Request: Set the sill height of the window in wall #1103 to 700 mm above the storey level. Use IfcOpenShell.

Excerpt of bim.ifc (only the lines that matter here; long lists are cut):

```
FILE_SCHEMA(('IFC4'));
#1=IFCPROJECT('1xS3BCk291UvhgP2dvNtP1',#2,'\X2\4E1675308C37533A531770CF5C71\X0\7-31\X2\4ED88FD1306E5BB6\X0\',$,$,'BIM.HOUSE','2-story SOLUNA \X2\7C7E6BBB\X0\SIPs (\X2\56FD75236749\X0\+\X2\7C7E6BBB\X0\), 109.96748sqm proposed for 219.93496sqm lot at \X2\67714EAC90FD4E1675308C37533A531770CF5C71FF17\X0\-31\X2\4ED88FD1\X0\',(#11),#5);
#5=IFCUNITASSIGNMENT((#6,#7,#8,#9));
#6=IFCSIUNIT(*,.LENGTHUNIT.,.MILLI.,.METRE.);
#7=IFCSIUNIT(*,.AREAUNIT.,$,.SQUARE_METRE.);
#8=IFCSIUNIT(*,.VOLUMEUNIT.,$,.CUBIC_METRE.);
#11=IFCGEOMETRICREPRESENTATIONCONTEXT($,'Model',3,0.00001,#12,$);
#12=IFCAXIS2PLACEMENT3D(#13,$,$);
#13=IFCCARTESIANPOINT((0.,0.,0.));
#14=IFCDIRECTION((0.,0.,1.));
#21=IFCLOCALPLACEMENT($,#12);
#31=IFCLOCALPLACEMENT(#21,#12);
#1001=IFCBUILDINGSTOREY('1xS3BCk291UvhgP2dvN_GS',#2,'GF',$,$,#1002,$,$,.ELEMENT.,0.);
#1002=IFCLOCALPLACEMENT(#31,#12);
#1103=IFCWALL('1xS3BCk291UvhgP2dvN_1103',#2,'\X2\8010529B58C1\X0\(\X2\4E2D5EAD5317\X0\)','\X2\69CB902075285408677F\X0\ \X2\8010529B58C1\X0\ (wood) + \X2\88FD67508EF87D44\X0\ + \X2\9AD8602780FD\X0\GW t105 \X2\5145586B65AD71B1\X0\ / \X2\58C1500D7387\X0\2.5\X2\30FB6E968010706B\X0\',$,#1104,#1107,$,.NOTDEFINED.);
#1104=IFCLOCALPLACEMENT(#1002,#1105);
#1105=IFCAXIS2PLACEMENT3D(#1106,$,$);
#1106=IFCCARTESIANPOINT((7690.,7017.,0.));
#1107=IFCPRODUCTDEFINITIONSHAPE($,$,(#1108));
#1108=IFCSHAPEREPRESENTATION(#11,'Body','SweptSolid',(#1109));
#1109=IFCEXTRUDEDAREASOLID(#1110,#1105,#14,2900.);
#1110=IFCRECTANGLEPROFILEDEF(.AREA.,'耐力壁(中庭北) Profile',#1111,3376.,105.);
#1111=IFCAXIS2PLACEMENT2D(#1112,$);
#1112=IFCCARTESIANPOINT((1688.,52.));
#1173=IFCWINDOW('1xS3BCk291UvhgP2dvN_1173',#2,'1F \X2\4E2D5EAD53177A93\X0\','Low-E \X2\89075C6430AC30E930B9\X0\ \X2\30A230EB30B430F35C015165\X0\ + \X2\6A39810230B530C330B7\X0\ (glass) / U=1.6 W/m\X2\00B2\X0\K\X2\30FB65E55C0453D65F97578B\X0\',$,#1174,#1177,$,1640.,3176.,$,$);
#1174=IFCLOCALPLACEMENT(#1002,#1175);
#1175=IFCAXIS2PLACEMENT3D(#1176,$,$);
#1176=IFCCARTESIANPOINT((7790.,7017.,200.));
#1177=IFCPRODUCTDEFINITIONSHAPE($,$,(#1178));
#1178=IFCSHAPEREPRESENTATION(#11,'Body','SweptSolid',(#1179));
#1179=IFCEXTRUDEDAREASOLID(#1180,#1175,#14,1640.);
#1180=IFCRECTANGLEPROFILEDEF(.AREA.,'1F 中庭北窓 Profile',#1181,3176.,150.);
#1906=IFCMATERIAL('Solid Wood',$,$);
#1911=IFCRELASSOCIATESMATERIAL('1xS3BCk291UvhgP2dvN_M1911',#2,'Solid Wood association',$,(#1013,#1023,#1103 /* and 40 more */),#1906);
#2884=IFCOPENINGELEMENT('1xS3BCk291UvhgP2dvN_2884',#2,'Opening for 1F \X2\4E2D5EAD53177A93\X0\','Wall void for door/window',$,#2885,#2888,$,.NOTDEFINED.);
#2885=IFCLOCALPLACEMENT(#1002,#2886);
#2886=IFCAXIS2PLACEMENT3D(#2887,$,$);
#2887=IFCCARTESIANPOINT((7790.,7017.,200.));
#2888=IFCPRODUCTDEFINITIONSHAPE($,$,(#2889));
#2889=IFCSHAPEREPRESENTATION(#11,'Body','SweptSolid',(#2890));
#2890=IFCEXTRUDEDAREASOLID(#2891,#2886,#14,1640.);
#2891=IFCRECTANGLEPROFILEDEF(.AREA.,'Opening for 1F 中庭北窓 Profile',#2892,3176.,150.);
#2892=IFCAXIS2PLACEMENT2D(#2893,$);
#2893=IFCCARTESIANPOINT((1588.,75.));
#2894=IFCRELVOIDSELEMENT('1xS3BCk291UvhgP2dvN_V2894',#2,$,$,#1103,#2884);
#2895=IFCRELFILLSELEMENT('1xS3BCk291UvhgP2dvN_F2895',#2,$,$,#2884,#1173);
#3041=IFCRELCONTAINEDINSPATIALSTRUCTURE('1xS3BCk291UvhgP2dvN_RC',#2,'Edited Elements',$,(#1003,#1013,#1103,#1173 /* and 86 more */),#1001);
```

```python
import numpy as np
import ifcopenshell
import ifcopenshell.api.geometry
import ifcopenshell.geom
import ifcopenshell.util.element
import ifcopenshell.util.placement
import ifcopenshell.util.shape
import ifcopenshell.util.unit

model = ifcopenshell.open("bim.ifc")
unit_scale = ifcopenshell.util.unit.calculate_unit_scale(model)

window = model.by_guid("1xS3BCk291UvhgP2dvN_1173")
opening = window.FillsVoids[0].RelatingOpeningElement
storey = ifcopenshell.util.element.get_container(window, ifc_class="IfcBuildingStorey")
level = ifcopenshell.util.placement.get_local_placement(storey.ObjectPlacement)[2, 3]

# The opening's origin need not be at the sill, so measure its lowest point.
shape = ifcopenshell.geom.create_shape(ifcopenshell.geom.settings(), opening)
bottom = ifcopenshell.util.shape.get_shape_bottom_elevation(shape, shape.geometry) / unit_scale
dz = level + 0.7 / unit_scale - bottom

shift = np.array([0.0, 0.0, dz])
# The window is not placed relative to its opening, so move both.
for product in (opening, window):
    matrix = ifcopenshell.util.placement.get_local_placement(product.ObjectPlacement)
    matrix[:3, 3] += shift
    ifcopenshell.api.geometry.edit_object_placement(model, product=product, matrix=matrix, is_si=False)

print(f"moved by {dz * unit_scale:+.3f} m")

model.write("bim_edited.ifc")
```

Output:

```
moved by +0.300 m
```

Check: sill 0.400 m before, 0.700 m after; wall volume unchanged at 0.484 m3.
